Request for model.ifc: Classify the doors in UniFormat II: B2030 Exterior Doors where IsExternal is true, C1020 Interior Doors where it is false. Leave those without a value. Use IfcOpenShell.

First a look at what the model holds.

```python
import ifcopenshell
import ifcopenshell.util.element

model = ifcopenshell.open("model.ifc")
print(model.schema)
print("classifications:", [c.Name for c in model.by_type("IfcClassification")])
values = [ifcopenshell.util.element.get_pset(e, "Pset_DoorCommon", "IsExternal") for e in model.by_type("IfcDoor")]
for value in (True, False, None):
    print("IsExternal", value, values.count(value))
```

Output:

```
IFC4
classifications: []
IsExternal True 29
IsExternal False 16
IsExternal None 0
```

```python
import ifcopenshell
import ifcopenshell.api.classification
import ifcopenshell.util.element

model = ifcopenshell.open("model.ifc")

system = ifcopenshell.api.classification.add_classification(model, classification="UniFormat II")

doors = model.by_type("IfcDoor")
external = {e: ifcopenshell.util.element.get_pset(e, "Pset_DoorCommon", "IsExternal") for e in doors}
for flag, code, name in ((True, "B2030", "Exterior Doors"), (False, "C1020", "Interior Doors")):
    products = [e for e in doors if external[e] is flag]
    ifcopenshell.api.classification.add_reference(
        model, products=products, classification=system, identification=code, name=name
    )
    print(code, len(products))

model.write("model_rev.ifc")
```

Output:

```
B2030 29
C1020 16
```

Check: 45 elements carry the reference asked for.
